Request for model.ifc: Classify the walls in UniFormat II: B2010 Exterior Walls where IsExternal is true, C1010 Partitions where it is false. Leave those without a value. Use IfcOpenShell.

First a look at what the model holds.

```python
import ifcopenshell
import ifcopenshell.util.element

model = ifcopenshell.open("model.ifc")
print(model.schema)
print("classifications:", [c.Name for c in model.by_type("IfcClassification")])
values = [ifcopenshell.util.element.get_pset(e, "Pset_WallCommon", "IsExternal") for e in model.by_type("IfcWall")]
for value in (True, False, None):
    print("IsExternal", value, values.count(value))
```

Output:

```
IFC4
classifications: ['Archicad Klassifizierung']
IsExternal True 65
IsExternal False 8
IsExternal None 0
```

```python
import ifcopenshell
import ifcopenshell.api.classification
import ifcopenshell.util.element

model = ifcopenshell.open("model.ifc")

system = ifcopenshell.api.classification.add_classification(model, classification="UniFormat II")

walls = model.by_type("IfcWall")
external = {e: ifcopenshell.util.element.get_pset(e, "Pset_WallCommon", "IsExternal") for e in walls}
for flag, code, name in ((True, "B2010", "Exterior Walls"), (False, "C1010", "Partitions")):
    products = [e for e in walls if external[e] is flag]
    ifcopenshell.api.classification.add_reference(
        model, products=products, classification=system, identification=code, name=name
    )
    print(code, len(products))

model.write("model_v2.ifc")
```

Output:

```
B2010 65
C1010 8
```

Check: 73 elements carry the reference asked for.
